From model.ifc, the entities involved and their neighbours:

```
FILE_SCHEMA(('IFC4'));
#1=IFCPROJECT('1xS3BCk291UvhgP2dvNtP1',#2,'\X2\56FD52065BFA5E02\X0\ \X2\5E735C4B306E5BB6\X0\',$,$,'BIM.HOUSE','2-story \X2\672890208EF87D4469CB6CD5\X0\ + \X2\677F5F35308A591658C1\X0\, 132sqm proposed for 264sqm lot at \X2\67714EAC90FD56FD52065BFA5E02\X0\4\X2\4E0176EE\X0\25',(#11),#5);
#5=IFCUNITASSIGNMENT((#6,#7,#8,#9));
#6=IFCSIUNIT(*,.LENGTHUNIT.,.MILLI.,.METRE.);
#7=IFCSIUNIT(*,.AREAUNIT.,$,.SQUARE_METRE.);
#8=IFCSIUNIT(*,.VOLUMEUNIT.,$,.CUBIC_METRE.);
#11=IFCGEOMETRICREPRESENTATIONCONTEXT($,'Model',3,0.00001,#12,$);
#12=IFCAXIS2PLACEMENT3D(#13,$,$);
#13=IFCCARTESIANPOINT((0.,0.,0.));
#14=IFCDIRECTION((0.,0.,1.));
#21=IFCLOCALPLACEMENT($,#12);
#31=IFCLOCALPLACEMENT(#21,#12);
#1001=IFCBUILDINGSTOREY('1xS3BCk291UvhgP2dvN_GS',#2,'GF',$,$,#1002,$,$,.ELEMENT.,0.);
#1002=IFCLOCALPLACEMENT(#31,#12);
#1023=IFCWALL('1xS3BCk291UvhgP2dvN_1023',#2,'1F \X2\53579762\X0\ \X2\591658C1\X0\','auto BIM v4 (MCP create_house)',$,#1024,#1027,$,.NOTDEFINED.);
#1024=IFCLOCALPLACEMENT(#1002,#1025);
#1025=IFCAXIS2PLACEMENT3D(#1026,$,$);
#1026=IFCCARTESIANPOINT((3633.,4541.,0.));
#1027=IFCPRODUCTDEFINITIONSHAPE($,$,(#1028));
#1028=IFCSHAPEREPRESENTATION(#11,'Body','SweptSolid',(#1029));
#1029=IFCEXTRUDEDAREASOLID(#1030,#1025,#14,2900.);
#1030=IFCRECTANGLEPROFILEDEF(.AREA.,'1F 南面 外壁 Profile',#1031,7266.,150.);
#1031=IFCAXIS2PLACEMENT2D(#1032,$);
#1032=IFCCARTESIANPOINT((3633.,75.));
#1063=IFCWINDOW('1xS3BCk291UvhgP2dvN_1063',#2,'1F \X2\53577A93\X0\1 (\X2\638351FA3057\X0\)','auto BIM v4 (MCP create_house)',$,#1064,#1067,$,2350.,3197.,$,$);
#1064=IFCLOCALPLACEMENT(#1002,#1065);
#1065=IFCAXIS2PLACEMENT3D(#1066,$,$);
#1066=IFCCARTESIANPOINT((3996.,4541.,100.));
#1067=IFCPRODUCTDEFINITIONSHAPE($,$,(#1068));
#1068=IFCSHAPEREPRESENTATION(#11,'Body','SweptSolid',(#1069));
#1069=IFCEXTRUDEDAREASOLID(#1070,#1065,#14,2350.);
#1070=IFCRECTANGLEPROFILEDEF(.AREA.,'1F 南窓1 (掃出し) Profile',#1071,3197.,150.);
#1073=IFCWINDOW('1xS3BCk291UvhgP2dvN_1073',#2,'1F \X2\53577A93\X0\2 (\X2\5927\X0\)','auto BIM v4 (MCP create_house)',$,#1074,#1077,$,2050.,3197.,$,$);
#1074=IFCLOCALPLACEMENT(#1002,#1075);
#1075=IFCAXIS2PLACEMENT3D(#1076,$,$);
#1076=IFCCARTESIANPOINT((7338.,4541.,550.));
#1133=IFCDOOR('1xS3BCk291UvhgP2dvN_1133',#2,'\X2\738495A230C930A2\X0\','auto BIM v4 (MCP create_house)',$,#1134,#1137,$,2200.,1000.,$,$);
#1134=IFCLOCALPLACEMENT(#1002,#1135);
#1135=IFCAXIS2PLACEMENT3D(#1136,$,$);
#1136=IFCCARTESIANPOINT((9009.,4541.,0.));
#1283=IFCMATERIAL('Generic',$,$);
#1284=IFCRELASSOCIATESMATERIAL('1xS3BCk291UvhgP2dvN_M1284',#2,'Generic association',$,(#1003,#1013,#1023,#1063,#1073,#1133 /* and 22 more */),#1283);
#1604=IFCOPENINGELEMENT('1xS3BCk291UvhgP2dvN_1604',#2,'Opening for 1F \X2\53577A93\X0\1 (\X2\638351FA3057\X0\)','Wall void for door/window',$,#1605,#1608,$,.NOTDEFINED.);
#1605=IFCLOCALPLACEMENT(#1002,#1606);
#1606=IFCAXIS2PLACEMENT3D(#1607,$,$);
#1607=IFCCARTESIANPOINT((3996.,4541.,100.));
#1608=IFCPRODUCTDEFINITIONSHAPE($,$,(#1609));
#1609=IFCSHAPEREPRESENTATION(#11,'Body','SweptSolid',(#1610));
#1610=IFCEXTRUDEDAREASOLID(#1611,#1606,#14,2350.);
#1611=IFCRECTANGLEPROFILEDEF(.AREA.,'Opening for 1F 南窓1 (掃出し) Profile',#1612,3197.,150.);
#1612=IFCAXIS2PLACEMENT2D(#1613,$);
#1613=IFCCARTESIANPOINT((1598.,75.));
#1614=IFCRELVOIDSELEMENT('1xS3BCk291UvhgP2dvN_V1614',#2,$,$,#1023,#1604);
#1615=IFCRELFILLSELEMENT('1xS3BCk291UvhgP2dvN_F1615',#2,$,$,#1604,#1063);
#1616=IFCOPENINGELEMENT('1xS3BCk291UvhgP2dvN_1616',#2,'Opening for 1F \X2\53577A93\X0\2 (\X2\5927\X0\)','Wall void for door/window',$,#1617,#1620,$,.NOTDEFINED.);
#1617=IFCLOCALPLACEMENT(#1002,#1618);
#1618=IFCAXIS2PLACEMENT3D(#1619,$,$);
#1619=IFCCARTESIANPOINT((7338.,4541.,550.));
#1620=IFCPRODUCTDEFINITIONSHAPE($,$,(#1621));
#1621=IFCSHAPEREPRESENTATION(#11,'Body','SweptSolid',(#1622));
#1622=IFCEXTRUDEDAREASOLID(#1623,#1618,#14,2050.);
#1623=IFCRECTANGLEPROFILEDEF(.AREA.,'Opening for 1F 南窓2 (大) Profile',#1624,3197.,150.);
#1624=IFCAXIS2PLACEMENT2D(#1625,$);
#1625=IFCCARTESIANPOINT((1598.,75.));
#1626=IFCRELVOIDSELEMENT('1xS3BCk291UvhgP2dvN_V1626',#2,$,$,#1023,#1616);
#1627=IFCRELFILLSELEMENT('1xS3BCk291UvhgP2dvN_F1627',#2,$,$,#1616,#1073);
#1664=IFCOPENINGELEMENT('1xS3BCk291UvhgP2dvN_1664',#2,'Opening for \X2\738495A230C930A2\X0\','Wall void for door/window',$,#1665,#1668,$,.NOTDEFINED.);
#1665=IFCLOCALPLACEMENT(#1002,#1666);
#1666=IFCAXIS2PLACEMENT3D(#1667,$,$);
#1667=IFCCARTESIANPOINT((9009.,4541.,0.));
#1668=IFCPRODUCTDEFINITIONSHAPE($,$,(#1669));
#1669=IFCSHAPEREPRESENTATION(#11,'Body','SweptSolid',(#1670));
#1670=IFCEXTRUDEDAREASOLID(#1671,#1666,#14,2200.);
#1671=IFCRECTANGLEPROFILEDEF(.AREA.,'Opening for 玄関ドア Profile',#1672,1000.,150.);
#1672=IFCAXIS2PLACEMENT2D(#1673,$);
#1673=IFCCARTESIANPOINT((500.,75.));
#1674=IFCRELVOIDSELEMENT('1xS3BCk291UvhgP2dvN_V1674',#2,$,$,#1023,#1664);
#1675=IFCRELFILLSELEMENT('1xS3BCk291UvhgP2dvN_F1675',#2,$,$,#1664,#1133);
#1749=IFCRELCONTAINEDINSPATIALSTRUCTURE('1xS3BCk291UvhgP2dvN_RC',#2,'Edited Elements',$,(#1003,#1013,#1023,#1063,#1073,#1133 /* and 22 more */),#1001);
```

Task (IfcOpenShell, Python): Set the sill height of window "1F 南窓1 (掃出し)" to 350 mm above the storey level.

```python
import numpy as np
import ifcopenshell
import ifcopenshell.api.geometry
import ifcopenshell.geom
import ifcopenshell.util.element
import ifcopenshell.util.placement
import ifcopenshell.util.shape
import ifcopenshell.util.unit

model = ifcopenshell.open("model.ifc")
unit_scale = ifcopenshell.util.unit.calculate_unit_scale(model)

window = model.by_guid("1xS3BCk291UvhgP2dvN_1063")
opening = window.FillsVoids[0].RelatingOpeningElement
storey = ifcopenshell.util.element.get_container(window, ifc_class="IfcBuildingStorey")
level = ifcopenshell.util.placement.get_local_placement(storey.ObjectPlacement)[2, 3]

# The opening's origin need not be at the sill, so measure its lowest point.
shape = ifcopenshell.geom.create_shape(ifcopenshell.geom.settings(), opening)
bottom = ifcopenshell.util.shape.get_shape_bottom_elevation(shape, shape.geometry) / unit_scale
dz = level + 350.0 - bottom

shift = np.array([0.0, 0.0, dz])
# The window is not placed relative to its opening, so move both.
for product in (opening, window):
    matrix = ifcopenshell.util.placement.get_local_placement(product.ObjectPlacement)
    matrix[:3, 3] += shift
    ifcopenshell.api.geometry.edit_object_placement(model, product=product, matrix=matrix, is_si=False)

print(f"moved by {dz * unit_scale:+.3f} m")

model.write("model-out.ifc")
```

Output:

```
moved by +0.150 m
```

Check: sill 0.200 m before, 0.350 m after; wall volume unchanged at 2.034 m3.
